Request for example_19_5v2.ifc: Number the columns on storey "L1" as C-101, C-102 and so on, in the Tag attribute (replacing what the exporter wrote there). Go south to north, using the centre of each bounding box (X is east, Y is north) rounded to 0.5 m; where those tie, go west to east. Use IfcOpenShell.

First a look at what the model holds.

```python
import ifcopenshell
import ifcopenshell.util.element
import ifcopenshell.util.placement

model = ifcopenshell.open("example_19_5v2.ifc")
print(model.schema)
storey = next(s for s in model.by_type("IfcBuildingStorey") if s.Name == "L1")
columns = [e for e in ifcopenshell.util.element.get_decomposition(storey) if e.is_a("IfcColumn")]
for e in sorted(columns, key=lambda e: e.id()):
    origin = ifcopenshell.util.placement.get_local_placement(e.ObjectPlacement)[:3, 3]
    print(e.id(), e.Tag, e.Name, origin.round(2) + 0.0, sep=" | ")
```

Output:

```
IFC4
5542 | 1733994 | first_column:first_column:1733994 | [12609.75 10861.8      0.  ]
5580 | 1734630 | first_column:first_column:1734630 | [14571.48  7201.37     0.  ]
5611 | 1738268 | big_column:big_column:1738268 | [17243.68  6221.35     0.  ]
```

```python
import ifcopenshell
import ifcopenshell.geom
import ifcopenshell.util.element
import ifcopenshell.util.shape

model = ifcopenshell.open("example_19_5v2.ifc")
settings = ifcopenshell.geom.settings()
settings.set("use-world-coords", True)


def centre(element):
    shape = ifcopenshell.geom.create_shape(settings, element)
    return ifcopenshell.util.shape.get_bbox_centroid(shape.geometry)


storey = next(s for s in model.by_type("IfcBuildingStorey") if s.Name == "L1")
columns = [e for e in ifcopenshell.util.element.get_decomposition(storey) if e.is_a("IfcColumn")]

# Insertion points can sit at a corner or the storey origin, so sort by the geometry (in metres).
centres = {e: centre(e) for e in columns}
columns.sort(key=lambda e: (round(centres[e][1] / 0.5), centres[e][0]))

for i, e in enumerate(columns, start=1):
    number = f"C-1{i:02d}"
    e.Tag = number
    print(e.id(), number)

model.write("example_19_5v2_edited.ifc")
```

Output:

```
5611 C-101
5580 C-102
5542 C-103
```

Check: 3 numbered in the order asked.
